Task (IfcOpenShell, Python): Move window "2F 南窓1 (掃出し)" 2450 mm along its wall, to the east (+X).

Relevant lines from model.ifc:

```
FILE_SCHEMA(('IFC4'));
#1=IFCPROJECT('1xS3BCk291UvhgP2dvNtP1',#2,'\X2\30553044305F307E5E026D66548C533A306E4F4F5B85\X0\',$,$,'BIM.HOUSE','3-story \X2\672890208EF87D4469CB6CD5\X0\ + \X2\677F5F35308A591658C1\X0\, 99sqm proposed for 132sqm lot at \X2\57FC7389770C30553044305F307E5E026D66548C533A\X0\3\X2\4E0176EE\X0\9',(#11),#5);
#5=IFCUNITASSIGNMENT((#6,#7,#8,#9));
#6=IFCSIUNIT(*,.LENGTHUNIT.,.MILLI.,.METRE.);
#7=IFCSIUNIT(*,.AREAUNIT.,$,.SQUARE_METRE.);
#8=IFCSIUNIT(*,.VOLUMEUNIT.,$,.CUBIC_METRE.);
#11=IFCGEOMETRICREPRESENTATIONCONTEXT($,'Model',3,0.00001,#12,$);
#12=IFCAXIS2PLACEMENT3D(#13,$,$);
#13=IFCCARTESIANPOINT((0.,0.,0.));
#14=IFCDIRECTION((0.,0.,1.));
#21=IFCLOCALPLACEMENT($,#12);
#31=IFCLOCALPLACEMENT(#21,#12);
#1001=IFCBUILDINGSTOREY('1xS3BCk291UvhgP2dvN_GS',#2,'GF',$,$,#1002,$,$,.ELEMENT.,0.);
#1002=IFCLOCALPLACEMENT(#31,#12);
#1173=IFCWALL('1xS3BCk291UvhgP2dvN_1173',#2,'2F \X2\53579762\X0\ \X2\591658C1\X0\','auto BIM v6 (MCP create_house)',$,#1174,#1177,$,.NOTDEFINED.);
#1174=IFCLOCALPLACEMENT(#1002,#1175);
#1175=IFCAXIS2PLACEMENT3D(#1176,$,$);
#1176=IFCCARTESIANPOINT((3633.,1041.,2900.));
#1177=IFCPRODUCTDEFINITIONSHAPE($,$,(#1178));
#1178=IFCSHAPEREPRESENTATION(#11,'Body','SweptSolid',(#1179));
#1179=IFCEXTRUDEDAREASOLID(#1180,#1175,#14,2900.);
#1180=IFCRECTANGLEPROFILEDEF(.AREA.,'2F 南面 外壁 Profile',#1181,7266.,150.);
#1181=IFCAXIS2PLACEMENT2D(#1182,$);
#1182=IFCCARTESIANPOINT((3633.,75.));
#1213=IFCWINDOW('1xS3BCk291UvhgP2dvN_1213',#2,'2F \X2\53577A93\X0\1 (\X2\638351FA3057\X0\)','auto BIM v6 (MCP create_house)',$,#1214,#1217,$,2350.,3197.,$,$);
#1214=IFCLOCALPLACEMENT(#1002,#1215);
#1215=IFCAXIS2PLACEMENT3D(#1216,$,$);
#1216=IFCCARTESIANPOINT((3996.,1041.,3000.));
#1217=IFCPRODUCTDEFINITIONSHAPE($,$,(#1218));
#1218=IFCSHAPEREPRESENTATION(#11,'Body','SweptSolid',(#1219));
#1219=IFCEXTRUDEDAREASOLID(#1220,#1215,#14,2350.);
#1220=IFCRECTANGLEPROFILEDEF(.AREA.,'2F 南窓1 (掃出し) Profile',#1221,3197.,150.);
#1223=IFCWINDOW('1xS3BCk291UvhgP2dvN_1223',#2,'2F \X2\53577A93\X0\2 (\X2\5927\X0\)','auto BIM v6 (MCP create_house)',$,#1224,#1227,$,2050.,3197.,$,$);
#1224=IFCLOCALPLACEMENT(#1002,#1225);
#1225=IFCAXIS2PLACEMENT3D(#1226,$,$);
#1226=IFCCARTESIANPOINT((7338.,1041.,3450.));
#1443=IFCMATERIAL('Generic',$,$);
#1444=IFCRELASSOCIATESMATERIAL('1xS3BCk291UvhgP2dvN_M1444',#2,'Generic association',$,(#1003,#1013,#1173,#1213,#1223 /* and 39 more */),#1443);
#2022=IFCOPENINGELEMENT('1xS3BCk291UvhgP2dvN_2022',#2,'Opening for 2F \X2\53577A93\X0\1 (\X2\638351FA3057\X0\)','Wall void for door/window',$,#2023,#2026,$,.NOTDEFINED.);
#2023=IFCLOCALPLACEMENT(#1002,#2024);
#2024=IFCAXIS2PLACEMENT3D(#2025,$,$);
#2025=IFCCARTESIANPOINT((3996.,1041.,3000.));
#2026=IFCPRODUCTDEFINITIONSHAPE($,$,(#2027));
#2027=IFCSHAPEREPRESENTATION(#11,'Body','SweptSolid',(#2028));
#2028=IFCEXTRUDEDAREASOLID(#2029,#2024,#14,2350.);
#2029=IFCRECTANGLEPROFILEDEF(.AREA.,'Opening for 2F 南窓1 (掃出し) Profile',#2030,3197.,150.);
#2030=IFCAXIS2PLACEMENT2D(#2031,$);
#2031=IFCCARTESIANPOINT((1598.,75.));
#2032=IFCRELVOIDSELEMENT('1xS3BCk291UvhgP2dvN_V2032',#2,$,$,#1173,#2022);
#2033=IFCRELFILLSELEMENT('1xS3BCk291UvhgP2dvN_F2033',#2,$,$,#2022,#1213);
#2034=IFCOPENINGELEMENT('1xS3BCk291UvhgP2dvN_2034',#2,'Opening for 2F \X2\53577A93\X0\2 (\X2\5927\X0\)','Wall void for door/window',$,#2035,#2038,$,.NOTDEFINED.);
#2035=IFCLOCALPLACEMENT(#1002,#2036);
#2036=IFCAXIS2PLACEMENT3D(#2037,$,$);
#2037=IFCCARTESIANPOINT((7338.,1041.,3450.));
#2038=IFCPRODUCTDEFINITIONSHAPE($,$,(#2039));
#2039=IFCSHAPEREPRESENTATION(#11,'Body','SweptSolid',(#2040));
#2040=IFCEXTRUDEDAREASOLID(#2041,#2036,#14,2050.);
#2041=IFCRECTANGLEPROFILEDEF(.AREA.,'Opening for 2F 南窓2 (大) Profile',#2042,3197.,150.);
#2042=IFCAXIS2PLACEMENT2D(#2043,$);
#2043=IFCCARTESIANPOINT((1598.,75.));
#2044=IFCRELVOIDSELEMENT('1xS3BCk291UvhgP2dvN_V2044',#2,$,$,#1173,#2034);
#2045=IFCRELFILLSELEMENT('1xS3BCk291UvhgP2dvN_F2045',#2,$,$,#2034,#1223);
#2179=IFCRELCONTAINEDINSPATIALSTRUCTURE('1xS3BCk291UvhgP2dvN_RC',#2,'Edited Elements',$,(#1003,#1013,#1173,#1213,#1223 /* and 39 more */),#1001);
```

```python
import ifcopenshell
import ifcopenshell.api.geometry
import ifcopenshell.util.placement
import ifcopenshell.util.unit

model = ifcopenshell.open("model.ifc")
unit_scale = ifcopenshell.util.unit.calculate_unit_scale(model)

window = model.by_guid("1xS3BCk291UvhgP2dvN_1213")
opening = window.FillsVoids[0].RelatingOpeningElement
wall = opening.VoidsElements[0].RelatingBuildingElement

wall_matrix = ifcopenshell.util.placement.get_local_placement(wall.ObjectPlacement)
shift = wall_matrix[:3, 0] * 2.45 / unit_scale
before = ifcopenshell.util.placement.get_local_placement(window.ObjectPlacement)[:3, 3].copy()

# The window is not placed relative to its opening, so move both.
for product in (opening, window):
    matrix = ifcopenshell.util.placement.get_local_placement(product.ObjectPlacement)
    matrix[:3, 3] += shift
    ifcopenshell.api.geometry.edit_object_placement(model, product=product, matrix=matrix, is_si=False)

after = ifcopenshell.util.placement.get_local_placement(window.ObjectPlacement)[:3, 3]
print("window moved by", (after - before).round(3) + 0.0)

model.write("model_rev.ifc")
```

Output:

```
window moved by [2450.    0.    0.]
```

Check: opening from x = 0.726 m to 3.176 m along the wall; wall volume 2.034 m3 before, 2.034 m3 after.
